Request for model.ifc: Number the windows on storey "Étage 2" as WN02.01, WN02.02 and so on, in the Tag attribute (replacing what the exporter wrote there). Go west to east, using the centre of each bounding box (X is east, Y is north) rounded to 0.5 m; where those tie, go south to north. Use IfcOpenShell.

First a look at what the model holds.

```python
import ifcopenshell
import ifcopenshell.util.element
import ifcopenshell.util.placement

model = ifcopenshell.open("model.ifc")
print(model.schema)
storey = next(s for s in model.by_type("IfcBuildingStorey") if s.Name == "Étage 2")
windows = [e for e in ifcopenshell.util.element.get_decomposition(storey) if e.is_a("IfcWindow")]
for e in sorted(windows, key=lambda e: e.id()):
    origin = ifcopenshell.util.placement.get_local_placement(e.ObjectPlacement)[:3, 3]
    print(e.id(), e.Tag, e.Name, origin.round(2) + 0.0, sep=" | ")
```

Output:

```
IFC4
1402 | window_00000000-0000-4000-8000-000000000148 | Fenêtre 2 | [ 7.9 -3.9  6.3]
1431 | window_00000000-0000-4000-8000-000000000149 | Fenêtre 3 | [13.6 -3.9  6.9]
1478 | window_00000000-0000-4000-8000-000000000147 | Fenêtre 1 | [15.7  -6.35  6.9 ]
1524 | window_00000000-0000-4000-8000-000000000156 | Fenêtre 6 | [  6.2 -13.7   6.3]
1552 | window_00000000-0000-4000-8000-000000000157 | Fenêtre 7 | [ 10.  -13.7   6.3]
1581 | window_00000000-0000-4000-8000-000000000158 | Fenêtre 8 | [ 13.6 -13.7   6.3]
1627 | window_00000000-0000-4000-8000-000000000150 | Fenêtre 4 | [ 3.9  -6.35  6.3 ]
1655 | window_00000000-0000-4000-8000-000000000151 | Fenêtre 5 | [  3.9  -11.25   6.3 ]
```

```python
import ifcopenshell
import ifcopenshell.geom
import ifcopenshell.util.element
import ifcopenshell.util.shape

model = ifcopenshell.open("model.ifc")
settings = ifcopenshell.geom.settings()
settings.set("use-world-coords", True)


def centre(element):
    shape = ifcopenshell.geom.create_shape(settings, element)
    return ifcopenshell.util.shape.get_bbox_centroid(shape.geometry)


storey = next(s for s in model.by_type("IfcBuildingStorey") if s.Name == "Étage 2")
windows = [e for e in ifcopenshell.util.element.get_decomposition(storey) if e.is_a("IfcWindow")]

# Insertion points can sit at a corner or the storey origin, so sort by the geometry (in metres).
centres = {e: centre(e) for e in windows}
windows.sort(key=lambda e: (round(centres[e][0] / 0.5), centres[e][1]))

for i, e in enumerate(windows, start=1):
    number = f"WN02.{i:02d}"
    e.Tag = number
    print(e.id(), number)

model.write("model_edited.ifc")
```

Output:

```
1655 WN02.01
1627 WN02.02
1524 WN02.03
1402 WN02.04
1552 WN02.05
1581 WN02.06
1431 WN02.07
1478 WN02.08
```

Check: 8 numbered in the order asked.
